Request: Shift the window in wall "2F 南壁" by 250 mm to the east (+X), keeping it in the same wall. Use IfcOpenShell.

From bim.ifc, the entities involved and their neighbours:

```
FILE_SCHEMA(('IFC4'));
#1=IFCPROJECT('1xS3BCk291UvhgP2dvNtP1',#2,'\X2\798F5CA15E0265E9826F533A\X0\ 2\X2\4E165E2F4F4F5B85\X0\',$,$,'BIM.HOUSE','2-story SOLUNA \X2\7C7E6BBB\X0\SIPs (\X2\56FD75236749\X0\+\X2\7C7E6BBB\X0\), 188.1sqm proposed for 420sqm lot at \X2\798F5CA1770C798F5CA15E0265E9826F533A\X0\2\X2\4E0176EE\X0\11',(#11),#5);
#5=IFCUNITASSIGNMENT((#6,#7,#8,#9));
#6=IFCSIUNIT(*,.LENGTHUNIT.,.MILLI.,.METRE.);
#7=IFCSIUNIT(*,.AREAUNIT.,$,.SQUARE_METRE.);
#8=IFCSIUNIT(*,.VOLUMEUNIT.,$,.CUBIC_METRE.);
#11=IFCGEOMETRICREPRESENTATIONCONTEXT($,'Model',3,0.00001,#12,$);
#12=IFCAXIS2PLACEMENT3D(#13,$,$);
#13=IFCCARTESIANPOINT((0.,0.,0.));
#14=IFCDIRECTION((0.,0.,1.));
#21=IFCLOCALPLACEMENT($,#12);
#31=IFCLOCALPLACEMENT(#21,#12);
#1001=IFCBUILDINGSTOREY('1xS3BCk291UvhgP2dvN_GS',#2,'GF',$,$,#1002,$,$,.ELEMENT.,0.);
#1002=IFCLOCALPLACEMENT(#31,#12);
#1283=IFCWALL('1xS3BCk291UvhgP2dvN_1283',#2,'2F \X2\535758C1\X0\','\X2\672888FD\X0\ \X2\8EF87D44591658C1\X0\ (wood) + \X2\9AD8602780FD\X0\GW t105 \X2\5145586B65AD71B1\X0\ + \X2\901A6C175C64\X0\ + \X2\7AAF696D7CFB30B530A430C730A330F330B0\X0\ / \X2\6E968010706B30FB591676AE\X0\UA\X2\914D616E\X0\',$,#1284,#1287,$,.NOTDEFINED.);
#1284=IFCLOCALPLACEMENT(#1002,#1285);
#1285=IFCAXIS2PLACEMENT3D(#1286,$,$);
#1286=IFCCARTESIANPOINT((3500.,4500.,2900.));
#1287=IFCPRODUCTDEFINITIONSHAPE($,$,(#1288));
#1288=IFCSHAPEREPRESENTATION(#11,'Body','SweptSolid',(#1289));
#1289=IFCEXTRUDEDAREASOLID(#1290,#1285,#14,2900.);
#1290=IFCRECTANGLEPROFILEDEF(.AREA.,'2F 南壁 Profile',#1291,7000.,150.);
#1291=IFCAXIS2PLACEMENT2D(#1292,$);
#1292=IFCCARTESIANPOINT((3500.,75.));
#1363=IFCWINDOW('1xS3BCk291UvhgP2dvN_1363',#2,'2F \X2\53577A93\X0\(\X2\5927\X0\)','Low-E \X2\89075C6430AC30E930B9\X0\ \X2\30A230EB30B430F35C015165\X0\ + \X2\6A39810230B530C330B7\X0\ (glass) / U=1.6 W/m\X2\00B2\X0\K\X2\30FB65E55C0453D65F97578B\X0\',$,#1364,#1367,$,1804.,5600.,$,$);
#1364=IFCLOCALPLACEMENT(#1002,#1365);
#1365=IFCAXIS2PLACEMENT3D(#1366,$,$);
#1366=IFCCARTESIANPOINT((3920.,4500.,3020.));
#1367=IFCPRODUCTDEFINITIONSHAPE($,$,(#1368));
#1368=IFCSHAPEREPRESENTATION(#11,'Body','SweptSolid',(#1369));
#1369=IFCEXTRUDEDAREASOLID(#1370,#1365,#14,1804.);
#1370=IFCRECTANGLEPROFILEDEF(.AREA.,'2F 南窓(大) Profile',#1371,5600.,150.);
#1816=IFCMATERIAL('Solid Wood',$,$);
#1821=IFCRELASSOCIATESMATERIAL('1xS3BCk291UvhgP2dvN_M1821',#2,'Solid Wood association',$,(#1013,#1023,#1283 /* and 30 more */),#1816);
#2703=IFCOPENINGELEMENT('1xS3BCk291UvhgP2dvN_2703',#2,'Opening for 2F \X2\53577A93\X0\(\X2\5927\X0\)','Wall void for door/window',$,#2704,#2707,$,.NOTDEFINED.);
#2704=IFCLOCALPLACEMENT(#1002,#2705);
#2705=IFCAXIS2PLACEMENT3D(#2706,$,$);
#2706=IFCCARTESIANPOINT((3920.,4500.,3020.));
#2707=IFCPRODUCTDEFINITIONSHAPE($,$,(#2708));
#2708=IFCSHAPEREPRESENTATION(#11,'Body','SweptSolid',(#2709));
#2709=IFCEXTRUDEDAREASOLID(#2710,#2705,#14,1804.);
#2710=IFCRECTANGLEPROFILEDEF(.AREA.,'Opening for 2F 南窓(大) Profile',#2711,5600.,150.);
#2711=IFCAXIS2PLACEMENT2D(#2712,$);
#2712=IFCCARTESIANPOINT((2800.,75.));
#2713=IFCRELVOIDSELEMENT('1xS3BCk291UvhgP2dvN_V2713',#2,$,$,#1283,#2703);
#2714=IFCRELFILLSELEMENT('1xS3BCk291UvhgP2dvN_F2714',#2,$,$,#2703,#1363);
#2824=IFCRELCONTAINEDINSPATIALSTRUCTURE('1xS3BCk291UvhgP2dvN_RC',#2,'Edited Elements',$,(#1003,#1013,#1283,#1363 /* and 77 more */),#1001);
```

```python
import ifcopenshell
import ifcopenshell.api.geometry
import ifcopenshell.util.placement
import ifcopenshell.util.unit

model = ifcopenshell.open("bim.ifc")
unit_scale = ifcopenshell.util.unit.calculate_unit_scale(model)

window = model.by_id(1363)
opening = window.FillsVoids[0].RelatingOpeningElement
wall = opening.VoidsElements[0].RelatingBuildingElement

wall_matrix = ifcopenshell.util.placement.get_local_placement(wall.ObjectPlacement)
shift = wall_matrix[:3, 0] * 0.25 / unit_scale
before = ifcopenshell.util.placement.get_local_placement(window.ObjectPlacement)[:3, 3].copy()

# The window is not placed relative to its opening, so move both.
for product in (opening, window):
    matrix = ifcopenshell.util.placement.get_local_placement(product.ObjectPlacement)
    matrix[:3, 3] += shift
    ifcopenshell.api.geometry.edit_object_placement(model, product=product, matrix=matrix, is_si=False)

after = ifcopenshell.util.placement.get_local_placement(window.ObjectPlacement)[:3, 3]
print("window moved by", (after - before).round(3) + 0.0)

model.write("bim_v2.ifc")
```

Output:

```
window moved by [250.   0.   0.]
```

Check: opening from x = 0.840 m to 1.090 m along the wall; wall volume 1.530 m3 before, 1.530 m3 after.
